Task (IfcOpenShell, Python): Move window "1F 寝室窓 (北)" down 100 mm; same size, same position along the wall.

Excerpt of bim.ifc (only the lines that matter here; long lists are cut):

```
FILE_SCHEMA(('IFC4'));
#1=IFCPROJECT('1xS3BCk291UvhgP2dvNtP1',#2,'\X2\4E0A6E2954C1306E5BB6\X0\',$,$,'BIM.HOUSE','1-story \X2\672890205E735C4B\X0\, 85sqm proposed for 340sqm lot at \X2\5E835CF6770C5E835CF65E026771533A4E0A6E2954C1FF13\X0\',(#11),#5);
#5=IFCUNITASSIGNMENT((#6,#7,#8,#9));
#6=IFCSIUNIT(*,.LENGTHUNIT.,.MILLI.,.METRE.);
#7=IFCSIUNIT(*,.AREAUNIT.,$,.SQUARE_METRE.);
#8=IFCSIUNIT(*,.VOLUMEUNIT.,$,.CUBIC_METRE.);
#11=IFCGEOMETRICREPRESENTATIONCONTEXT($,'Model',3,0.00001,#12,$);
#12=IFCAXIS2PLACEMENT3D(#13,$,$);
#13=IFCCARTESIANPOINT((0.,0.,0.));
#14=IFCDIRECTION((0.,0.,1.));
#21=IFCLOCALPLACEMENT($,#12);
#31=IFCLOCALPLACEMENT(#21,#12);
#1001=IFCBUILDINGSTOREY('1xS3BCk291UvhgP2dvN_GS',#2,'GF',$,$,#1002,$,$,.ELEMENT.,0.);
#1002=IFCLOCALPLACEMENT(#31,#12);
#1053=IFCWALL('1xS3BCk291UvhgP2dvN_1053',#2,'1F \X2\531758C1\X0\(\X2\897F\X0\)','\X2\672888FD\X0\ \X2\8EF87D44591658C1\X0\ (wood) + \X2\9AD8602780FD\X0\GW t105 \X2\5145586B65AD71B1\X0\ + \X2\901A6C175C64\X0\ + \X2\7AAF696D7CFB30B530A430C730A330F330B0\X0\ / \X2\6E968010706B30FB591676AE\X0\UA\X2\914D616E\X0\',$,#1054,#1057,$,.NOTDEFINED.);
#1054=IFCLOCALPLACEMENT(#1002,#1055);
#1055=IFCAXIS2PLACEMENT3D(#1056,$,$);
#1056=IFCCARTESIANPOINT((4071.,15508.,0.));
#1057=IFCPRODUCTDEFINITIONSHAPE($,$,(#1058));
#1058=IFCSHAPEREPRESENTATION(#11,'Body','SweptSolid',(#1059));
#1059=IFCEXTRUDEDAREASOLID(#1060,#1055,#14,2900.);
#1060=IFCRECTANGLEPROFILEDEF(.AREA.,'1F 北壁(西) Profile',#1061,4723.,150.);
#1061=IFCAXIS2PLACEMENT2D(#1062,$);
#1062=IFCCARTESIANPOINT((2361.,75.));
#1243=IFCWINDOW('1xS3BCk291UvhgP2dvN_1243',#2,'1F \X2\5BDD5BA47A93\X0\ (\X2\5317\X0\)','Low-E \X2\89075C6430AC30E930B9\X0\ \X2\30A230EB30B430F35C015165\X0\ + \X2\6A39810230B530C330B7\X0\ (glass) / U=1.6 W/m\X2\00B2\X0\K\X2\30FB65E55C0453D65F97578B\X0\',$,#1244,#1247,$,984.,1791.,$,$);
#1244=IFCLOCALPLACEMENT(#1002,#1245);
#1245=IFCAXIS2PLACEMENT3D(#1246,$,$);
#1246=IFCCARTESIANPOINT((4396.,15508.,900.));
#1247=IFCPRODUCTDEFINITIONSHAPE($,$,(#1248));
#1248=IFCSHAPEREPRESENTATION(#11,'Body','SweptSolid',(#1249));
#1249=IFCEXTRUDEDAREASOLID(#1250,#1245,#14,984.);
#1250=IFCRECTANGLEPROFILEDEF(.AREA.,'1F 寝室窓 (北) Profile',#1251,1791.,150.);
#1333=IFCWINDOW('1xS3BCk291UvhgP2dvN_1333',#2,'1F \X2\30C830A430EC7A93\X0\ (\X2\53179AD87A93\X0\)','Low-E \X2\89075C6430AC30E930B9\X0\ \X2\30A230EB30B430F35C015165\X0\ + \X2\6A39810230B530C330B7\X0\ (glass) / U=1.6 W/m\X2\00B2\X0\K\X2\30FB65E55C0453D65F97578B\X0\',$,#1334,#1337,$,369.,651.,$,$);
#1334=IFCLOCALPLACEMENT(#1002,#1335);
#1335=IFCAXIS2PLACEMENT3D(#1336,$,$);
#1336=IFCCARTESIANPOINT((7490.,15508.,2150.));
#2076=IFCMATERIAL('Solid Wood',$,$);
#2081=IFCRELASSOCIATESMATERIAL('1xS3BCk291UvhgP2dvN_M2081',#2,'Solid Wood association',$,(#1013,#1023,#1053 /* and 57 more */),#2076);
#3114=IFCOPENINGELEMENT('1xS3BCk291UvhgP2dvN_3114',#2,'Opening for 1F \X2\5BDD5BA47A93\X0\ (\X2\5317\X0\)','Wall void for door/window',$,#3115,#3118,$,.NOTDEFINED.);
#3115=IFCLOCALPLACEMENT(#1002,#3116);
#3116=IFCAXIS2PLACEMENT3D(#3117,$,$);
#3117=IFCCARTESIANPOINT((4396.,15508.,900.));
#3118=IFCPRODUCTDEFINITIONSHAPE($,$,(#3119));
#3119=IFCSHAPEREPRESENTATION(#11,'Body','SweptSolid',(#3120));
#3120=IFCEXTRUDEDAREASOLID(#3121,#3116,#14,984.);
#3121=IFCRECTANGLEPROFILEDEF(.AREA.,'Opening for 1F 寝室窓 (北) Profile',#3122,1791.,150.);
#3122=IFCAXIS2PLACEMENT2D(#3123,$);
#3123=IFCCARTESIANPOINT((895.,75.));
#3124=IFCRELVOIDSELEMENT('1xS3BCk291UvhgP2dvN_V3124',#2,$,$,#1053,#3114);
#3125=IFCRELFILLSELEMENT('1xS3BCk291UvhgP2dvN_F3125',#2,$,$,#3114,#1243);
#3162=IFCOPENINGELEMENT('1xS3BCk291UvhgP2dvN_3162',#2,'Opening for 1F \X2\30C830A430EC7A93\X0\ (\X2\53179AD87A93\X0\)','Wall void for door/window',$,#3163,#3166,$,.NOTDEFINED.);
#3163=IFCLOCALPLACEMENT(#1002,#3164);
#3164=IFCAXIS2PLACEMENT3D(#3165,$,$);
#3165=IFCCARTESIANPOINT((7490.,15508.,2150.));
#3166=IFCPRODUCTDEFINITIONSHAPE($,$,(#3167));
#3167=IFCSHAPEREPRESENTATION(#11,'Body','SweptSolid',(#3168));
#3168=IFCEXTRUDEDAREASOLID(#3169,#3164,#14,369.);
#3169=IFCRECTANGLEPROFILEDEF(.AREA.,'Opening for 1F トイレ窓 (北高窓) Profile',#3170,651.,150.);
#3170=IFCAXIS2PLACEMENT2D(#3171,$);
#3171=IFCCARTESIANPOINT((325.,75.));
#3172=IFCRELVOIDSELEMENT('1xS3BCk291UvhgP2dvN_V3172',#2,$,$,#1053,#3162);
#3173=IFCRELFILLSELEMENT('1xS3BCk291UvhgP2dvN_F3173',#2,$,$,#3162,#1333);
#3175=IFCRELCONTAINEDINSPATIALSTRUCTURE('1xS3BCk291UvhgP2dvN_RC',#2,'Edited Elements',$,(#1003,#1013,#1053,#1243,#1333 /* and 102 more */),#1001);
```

```python
import numpy as np
import ifcopenshell
import ifcopenshell.api.geometry
import ifcopenshell.util.placement
import ifcopenshell.util.unit

model = ifcopenshell.open("bim.ifc")
unit_scale = ifcopenshell.util.unit.calculate_unit_scale(model)

window = model.by_guid("1xS3BCk291UvhgP2dvN_1243")
opening = window.FillsVoids[0].RelatingOpeningElement
dz = -0.1 / unit_scale

shift = np.array([0.0, 0.0, dz])
# The window is not placed relative to its opening, so move both.
for product in (opening, window):
    matrix = ifcopenshell.util.placement.get_local_placement(product.ObjectPlacement)
    matrix[:3, 3] += shift
    ifcopenshell.api.geometry.edit_object_placement(model, product=product, matrix=matrix, is_si=False)

print(f"moved by {dz * unit_scale:+.3f} m")

model.write("bim_edited.ifc")
```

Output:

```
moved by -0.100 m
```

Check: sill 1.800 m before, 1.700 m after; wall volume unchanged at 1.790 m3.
